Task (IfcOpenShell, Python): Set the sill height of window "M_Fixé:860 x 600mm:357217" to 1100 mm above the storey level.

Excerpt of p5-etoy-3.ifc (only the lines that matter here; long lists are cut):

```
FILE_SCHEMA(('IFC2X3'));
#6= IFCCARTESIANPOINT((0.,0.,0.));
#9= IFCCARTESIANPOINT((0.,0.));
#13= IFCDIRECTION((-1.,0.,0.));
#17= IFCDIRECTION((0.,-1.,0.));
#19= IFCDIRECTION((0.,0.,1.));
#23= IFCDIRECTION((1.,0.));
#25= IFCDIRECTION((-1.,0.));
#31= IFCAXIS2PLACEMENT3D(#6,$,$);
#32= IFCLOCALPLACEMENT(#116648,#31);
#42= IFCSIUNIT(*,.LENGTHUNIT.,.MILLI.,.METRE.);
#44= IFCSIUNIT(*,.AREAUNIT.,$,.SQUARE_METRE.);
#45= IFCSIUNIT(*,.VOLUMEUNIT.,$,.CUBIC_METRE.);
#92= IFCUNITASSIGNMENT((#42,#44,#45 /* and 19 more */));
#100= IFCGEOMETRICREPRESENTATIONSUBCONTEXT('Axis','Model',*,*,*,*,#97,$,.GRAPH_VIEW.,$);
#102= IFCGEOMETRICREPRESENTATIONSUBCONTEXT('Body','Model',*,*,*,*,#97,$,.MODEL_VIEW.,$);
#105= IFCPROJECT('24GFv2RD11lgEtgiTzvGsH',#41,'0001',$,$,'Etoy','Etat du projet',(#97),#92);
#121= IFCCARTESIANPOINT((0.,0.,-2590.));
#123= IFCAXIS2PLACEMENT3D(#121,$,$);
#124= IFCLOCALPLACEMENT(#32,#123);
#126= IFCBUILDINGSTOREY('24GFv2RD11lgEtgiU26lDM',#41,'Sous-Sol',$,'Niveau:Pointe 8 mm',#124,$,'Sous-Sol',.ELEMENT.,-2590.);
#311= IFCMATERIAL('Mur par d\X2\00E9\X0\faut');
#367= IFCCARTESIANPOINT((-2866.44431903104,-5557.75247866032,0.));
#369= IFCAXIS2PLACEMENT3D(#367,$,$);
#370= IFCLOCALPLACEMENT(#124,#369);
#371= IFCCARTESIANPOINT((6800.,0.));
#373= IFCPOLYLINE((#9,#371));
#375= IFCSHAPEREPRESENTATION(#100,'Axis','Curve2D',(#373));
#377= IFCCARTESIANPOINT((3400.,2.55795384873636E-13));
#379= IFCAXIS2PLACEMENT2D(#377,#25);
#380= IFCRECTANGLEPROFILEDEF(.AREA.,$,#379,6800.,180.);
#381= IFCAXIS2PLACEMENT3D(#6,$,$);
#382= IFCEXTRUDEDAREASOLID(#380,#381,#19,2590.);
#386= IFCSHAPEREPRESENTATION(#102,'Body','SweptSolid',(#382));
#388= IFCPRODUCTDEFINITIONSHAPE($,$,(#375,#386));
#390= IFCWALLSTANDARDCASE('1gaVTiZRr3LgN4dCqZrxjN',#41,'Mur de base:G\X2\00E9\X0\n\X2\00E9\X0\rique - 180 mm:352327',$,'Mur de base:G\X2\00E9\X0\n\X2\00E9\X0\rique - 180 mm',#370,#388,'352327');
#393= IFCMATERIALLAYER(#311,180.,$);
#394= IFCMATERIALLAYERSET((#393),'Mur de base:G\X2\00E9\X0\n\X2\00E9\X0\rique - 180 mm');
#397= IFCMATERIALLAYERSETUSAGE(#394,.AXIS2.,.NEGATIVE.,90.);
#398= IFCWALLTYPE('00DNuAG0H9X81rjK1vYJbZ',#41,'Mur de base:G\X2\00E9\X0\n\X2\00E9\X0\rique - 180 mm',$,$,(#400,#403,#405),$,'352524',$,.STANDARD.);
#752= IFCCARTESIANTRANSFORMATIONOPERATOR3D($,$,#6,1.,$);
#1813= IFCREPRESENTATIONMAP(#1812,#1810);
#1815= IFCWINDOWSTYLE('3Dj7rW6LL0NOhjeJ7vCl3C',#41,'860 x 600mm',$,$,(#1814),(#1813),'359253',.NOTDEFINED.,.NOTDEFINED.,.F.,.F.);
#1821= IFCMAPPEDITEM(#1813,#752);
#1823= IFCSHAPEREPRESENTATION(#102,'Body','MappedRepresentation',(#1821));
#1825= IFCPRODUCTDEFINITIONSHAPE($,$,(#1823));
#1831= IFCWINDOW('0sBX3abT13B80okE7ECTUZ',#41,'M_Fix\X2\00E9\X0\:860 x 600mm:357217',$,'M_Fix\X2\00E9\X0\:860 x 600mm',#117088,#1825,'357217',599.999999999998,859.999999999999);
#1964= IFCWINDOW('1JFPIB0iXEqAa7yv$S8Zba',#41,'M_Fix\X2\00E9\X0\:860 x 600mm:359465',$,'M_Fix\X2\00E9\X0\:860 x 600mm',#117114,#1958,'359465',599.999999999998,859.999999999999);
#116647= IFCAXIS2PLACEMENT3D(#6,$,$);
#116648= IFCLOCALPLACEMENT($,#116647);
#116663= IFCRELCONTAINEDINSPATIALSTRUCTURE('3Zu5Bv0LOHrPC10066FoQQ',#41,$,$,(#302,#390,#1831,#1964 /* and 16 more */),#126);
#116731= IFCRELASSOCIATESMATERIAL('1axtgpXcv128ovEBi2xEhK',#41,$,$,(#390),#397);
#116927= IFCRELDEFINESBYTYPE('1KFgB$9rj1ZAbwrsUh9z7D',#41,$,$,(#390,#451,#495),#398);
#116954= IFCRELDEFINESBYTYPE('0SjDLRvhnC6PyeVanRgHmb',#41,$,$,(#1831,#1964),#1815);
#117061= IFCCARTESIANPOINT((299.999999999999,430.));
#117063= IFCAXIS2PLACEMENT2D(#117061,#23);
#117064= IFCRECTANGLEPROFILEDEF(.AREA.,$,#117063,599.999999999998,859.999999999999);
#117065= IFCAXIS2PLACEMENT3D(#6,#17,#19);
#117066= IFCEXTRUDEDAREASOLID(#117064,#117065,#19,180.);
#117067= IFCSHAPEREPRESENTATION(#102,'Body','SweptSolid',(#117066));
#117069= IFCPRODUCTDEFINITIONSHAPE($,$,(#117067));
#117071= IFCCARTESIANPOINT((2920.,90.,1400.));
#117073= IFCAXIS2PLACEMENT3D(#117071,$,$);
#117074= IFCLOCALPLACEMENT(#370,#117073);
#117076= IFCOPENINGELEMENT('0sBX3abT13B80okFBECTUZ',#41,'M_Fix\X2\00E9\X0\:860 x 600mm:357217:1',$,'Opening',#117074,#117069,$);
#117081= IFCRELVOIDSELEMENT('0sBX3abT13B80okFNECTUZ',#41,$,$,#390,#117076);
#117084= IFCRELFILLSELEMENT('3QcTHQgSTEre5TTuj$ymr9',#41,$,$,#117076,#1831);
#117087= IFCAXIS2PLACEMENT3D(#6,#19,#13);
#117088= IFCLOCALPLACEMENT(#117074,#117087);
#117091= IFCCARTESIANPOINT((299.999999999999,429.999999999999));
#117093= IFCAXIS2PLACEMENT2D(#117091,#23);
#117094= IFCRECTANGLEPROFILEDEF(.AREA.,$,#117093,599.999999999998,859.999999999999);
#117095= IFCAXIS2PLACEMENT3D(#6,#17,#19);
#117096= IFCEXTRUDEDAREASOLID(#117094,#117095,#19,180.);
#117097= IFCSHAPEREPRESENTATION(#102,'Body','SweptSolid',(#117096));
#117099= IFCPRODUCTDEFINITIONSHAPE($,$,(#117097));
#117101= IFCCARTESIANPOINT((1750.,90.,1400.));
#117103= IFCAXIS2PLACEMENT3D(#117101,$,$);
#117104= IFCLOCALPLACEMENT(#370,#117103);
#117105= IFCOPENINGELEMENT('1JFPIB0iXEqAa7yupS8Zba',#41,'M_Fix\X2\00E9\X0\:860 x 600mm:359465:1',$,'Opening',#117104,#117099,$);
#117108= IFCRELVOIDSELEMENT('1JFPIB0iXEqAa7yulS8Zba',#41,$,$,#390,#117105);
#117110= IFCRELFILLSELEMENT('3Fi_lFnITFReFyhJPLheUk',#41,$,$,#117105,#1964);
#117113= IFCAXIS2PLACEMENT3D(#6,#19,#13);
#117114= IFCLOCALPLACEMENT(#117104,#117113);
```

```python
import numpy as np
import ifcopenshell
import ifcopenshell.api.geometry
import ifcopenshell.geom
import ifcopenshell.util.element
import ifcopenshell.util.placement
import ifcopenshell.util.shape
import ifcopenshell.util.unit

model = ifcopenshell.open("p5-etoy-3.ifc")
unit_scale = ifcopenshell.util.unit.calculate_unit_scale(model)

window = model.by_guid("0sBX3abT13B80okE7ECTUZ")
opening = window.FillsVoids[0].RelatingOpeningElement
storey = ifcopenshell.util.element.get_container(window, ifc_class="IfcBuildingStorey")
level = ifcopenshell.util.placement.get_local_placement(storey.ObjectPlacement)[2, 3]

# The opening's origin need not be at the sill, so measure its lowest point.
shape = ifcopenshell.geom.create_shape(ifcopenshell.geom.settings(), opening)
bottom = ifcopenshell.util.shape.get_shape_bottom_elevation(shape, shape.geometry) / unit_scale
dz = level + 1.1 / unit_scale - bottom

shift = np.array([0.0, 0.0, dz])
# The window is placed relative to its opening, so it follows when the opening moves.
matrix = ifcopenshell.util.placement.get_local_placement(opening.ObjectPlacement)
matrix[:3, 3] += shift
ifcopenshell.api.geometry.edit_object_placement(
    model, product=opening, matrix=matrix, is_si=False, should_transform_children=True
)

print(f"moved by {dz * unit_scale:+.3f} m")

model.write("p5-etoy-3-out.ifc")
```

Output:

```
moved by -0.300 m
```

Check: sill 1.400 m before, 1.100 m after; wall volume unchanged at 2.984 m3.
